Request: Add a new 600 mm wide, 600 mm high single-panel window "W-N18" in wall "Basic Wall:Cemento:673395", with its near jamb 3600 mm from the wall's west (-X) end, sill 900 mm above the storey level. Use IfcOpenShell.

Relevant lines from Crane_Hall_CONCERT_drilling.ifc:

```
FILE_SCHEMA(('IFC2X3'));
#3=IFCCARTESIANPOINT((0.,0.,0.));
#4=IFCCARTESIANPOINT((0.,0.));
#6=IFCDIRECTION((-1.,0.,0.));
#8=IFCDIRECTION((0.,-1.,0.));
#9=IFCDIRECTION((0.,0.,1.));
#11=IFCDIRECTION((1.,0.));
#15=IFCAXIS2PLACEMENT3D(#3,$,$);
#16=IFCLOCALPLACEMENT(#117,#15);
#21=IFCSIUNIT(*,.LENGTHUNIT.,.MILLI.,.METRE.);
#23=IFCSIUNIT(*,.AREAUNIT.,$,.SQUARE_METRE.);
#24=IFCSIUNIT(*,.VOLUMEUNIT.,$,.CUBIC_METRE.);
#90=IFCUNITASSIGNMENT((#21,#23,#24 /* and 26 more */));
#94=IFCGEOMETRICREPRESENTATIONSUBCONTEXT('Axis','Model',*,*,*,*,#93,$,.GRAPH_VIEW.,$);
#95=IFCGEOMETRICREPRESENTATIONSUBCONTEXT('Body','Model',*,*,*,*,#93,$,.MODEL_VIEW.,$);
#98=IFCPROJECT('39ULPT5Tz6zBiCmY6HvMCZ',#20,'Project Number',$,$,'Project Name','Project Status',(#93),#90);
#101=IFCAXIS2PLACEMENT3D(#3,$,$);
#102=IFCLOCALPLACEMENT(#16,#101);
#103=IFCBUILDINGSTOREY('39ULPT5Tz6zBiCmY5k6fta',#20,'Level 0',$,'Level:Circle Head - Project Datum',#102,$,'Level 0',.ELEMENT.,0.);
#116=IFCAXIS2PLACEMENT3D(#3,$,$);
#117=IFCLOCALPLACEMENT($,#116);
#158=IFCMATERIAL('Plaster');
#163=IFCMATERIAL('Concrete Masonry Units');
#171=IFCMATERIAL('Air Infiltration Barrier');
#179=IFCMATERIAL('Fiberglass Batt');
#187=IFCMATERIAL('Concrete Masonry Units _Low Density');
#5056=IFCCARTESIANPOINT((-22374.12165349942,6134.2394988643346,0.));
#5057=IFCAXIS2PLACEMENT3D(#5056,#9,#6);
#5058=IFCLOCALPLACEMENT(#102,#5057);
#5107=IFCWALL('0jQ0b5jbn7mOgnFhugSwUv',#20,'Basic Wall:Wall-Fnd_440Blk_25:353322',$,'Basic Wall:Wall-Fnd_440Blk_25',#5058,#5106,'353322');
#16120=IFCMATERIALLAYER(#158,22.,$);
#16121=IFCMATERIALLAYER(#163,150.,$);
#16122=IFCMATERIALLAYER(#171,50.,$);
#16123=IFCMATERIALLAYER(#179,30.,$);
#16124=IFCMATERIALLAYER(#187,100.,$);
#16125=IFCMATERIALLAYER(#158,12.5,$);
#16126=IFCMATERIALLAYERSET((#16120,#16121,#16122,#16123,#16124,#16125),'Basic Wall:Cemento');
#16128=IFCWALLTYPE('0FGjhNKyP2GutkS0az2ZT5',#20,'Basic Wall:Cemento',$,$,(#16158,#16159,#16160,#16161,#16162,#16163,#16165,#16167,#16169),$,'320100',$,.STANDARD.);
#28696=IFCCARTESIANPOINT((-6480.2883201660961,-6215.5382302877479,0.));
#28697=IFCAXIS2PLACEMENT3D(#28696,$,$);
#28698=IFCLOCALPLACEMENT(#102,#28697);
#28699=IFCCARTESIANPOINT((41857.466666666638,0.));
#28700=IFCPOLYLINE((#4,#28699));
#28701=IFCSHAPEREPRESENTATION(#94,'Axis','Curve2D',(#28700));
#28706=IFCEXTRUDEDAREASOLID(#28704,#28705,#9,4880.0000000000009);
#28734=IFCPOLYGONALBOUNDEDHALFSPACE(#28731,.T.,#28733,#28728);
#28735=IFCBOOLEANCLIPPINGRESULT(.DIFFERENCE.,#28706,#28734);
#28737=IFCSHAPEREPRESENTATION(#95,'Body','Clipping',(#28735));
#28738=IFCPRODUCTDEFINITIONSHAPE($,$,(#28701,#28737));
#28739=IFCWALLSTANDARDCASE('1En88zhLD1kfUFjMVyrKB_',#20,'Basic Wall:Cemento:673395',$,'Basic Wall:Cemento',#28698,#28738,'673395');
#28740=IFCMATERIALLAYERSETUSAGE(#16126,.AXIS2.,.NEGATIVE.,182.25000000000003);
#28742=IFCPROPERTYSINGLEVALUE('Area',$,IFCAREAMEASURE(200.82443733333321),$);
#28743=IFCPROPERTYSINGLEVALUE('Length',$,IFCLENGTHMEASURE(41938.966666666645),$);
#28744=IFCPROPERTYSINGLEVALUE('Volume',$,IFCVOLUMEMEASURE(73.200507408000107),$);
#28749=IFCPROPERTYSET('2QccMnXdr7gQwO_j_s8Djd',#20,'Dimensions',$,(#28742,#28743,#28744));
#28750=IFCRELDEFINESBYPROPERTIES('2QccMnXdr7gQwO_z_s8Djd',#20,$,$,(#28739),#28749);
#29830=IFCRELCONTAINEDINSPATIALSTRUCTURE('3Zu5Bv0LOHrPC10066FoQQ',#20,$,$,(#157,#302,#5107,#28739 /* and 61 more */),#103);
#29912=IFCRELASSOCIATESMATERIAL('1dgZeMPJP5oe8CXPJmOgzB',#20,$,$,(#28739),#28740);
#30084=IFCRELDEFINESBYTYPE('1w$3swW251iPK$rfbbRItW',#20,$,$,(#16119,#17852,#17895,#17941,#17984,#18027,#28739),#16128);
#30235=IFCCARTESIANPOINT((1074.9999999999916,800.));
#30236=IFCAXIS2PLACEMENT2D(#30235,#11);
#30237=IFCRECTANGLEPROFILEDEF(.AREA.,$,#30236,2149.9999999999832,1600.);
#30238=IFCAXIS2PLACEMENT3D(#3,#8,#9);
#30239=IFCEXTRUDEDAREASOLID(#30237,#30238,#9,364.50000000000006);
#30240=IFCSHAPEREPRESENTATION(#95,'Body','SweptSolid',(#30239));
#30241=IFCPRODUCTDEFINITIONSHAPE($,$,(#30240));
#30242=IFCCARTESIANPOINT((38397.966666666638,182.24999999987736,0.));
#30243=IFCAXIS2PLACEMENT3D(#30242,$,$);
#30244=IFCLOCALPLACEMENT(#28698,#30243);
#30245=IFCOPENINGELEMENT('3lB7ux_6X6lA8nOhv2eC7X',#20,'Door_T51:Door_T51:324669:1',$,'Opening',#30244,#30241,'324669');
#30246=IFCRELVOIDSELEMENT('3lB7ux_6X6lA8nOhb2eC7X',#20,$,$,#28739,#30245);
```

```python
import numpy as np
import ifcopenshell
import ifcopenshell.api.feature
import ifcopenshell.api.geometry
import ifcopenshell.api.pset
import ifcopenshell.api.root
import ifcopenshell.api.spatial
import ifcopenshell.api.type
import ifcopenshell.geom
import ifcopenshell.util.element
import ifcopenshell.util.placement
import ifcopenshell.util.representation
import ifcopenshell.util.shape
import ifcopenshell.util.unit

model = ifcopenshell.open("Crane_Hall_CONCERT_drilling.ifc")
unit_scale = ifcopenshell.util.unit.calculate_unit_scale(model)
area_scale = ifcopenshell.util.unit.calculate_unit_scale(model, "AREAUNIT")
volume_scale = ifcopenshell.util.unit.calculate_unit_scale(model, "VOLUMEUNIT")
settings = ifcopenshell.geom.settings()


def volume(element):
    """Net volume in cubic metres, openings subtracted."""
    shape = ifcopenshell.geom.create_shape(settings, element)
    return ifcopenshell.util.shape.get_volume(shape.geometry)


wall = model.by_guid("1En88zhLD1kfUFjMVyrKB_")
storey = ifcopenshell.util.element.get_container(wall, ifc_class="IfcBuildingStorey")
context = ifcopenshell.util.representation.get_context(model, "Model", "Body", "MODEL_VIEW")
before = volume(wall)

width, height, from_end, sill = 0.6, 0.6, 3.6, 0.9  # metres

# The wall runs along its own X axis, and the end named is its -X end.
wall_shape = ifcopenshell.geom.create_shape(settings, wall)
x, y, z = ifcopenshell.util.shape.get_vertices(wall_shape.geometry).T
start = x.min() + from_end
face, thickness = float(y.min()), float(y.max() - y.min())
wall_matrix = ifcopenshell.util.placement.get_local_placement(wall.ObjectPlacement)
level = ifcopenshell.util.placement.get_local_placement(storey.ObjectPlacement)[2, 3]


def in_wall(x, y):
    """Placement at x, y metres in the wall's axes, at sill height."""
    matrix = wall_matrix.copy()
    matrix[:, 3] = wall_matrix @ np.array([x / unit_scale, y / unit_scale, 0.0, 1.0])
    matrix[2, 3] = level + sill / unit_scale
    return matrix


# Opening: a box that overshoots both wall faces by 50 mm.
opening = ifcopenshell.api.root.create_entity(model, ifc_class="IfcOpeningElement")
box = ifcopenshell.api.geometry.add_wall_representation(
    model, context=context, length=width, height=height, thickness=thickness + 0.1
)
ifcopenshell.api.geometry.assign_representation(model, product=opening, representation=box)
ifcopenshell.api.geometry.edit_object_placement(model, product=opening, matrix=in_wall(start, face - 0.05), is_si=False)
ifcopenshell.api.feature.add_feature(model, feature=opening, element=wall)

window = ifcopenshell.api.root.create_entity(model, ifc_class="IfcWindow", name="W-N18")
window.OverallWidth, window.OverallHeight = width / unit_scale, height / unit_scale
body = ifcopenshell.api.geometry.add_window_representation(
    model,
    context=context,
    overall_width=window.OverallWidth,
    overall_height=window.OverallHeight,
    partition_type="SINGLE_PANEL",
)
ifcopenshell.api.geometry.assign_representation(model, product=window, representation=body)
ifcopenshell.api.spatial.assign_container(model, products=[window], relating_structure=storey)
fills = ifcopenshell.api.feature.add_filling(model, opening=opening, element=window)
fills.OwnerHistory = window.OwnerHistory  # required in IFC2X3

# IFC2X3 keeps the operation on the window style.
style = ifcopenshell.api.root.create_entity(model, ifc_class="IfcWindowStyle", name="W-N18")
style.OperationType, style.ConstructionType = "SINGLE_PANEL", "NOTDEFINED"
style.ParameterTakesPrecedence = style.Sizeable = False
ifcopenshell.api.type.assign_type(model, related_objects=[window], relating_type=style)

# Centre the window in the wall's thickness.
ifcopenshell.api.geometry.edit_object_placement(model, product=window, matrix=in_wall(start, face), is_si=False)
window_shape = ifcopenshell.geom.create_shape(settings, window)
depth = ifcopenshell.util.shape.get_vertices(window_shape.geometry)[:, 1]
offset = face + thickness / 2 - (depth.min() + depth.max()) / 2
ifcopenshell.api.geometry.edit_object_placement(model, product=window, matrix=in_wall(start, offset), is_si=False)

after = volume(wall)

# Update the wall's stored quantities.
pset = model.by_id(ifcopenshell.util.element.get_pset(wall, "Dimensions", should_inherit=False)["id"])
ifcopenshell.api.pset.edit_pset(model, pset=pset, properties={
    "Area": model.create_entity("IfcAreaMeasure", after / thickness / area_scale),
    "Volume": model.create_entity("IfcVolumeMeasure", after / volume_scale),
})

print(f"wall volume {before:.3f} -> {after:.3f} m3")

model.write("Crane_Hall_CONCERT_drilling-out.ifc")
```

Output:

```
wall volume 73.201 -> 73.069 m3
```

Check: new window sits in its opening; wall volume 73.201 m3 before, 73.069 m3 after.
